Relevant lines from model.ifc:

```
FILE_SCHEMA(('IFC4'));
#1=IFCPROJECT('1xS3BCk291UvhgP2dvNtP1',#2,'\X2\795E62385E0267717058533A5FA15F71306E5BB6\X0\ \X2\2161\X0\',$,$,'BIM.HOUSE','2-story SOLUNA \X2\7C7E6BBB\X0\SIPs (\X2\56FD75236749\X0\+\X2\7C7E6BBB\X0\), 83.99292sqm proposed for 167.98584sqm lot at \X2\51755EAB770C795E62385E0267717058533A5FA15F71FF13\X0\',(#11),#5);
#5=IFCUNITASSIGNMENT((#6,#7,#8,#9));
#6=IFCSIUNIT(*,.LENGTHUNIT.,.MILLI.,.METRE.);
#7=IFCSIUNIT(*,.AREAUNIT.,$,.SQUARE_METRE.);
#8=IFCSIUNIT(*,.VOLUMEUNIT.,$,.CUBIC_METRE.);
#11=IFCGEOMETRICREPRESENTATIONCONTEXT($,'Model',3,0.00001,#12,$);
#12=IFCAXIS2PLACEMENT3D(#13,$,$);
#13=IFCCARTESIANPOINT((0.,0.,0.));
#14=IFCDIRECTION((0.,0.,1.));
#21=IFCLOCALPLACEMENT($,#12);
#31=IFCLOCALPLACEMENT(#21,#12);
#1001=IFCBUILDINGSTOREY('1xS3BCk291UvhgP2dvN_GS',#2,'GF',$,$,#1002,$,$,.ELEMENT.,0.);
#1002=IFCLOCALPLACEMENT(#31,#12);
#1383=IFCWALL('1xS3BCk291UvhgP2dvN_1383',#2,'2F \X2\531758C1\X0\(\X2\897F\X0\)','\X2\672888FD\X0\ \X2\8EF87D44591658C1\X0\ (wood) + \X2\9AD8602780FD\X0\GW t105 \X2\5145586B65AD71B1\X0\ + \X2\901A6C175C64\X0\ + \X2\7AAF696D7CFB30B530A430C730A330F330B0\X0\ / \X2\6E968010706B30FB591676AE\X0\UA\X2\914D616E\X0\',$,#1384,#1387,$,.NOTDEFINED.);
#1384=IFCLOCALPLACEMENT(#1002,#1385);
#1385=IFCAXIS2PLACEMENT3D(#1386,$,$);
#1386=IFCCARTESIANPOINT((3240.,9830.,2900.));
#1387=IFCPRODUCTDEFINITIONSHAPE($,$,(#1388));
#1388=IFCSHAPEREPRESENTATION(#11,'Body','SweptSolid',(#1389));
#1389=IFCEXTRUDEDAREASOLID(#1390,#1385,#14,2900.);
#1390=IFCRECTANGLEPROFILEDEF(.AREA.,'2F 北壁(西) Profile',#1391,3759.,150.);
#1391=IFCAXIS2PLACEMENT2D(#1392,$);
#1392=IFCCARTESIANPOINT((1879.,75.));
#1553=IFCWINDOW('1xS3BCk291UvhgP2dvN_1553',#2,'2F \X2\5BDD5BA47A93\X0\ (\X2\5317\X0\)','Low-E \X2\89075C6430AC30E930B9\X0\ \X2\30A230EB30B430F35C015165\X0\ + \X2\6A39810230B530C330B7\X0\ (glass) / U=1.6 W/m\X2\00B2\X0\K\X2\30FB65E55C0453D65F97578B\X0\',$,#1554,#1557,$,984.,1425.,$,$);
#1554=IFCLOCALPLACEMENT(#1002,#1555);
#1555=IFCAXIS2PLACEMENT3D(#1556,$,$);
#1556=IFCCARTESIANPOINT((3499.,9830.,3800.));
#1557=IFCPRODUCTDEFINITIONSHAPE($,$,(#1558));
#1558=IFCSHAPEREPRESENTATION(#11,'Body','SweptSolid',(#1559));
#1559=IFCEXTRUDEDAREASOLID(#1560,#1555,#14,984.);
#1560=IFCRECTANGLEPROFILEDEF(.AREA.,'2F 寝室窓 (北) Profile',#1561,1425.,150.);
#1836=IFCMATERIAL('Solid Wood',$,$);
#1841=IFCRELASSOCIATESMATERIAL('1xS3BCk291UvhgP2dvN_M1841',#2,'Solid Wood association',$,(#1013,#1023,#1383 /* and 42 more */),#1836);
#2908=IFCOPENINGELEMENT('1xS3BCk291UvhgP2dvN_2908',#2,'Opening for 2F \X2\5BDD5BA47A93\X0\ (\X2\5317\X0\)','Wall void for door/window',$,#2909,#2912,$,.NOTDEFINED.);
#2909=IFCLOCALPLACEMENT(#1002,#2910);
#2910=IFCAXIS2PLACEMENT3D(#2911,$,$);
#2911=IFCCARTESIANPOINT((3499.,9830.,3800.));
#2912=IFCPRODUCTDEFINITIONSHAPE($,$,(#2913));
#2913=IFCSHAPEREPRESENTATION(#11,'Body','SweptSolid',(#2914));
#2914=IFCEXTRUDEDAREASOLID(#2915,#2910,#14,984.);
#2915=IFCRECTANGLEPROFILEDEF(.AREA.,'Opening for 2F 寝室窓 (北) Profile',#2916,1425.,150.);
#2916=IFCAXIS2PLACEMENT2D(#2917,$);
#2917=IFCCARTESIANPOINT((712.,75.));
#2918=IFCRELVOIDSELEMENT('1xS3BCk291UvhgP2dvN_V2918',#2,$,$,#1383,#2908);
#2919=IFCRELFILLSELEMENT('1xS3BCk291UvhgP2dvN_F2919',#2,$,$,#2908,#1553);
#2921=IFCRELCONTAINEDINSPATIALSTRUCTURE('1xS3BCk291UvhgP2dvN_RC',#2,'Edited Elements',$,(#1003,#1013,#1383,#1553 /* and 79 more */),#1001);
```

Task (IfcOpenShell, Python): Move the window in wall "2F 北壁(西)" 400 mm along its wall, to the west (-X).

```python
import ifcopenshell
import ifcopenshell.api.geometry
import ifcopenshell.util.placement
import ifcopenshell.util.unit

model = ifcopenshell.open("model.ifc")
unit_scale = ifcopenshell.util.unit.calculate_unit_scale(model)

window = model.by_guid("1xS3BCk291UvhgP2dvN_1553")
opening = window.FillsVoids[0].RelatingOpeningElement
wall = opening.VoidsElements[0].RelatingBuildingElement

wall_matrix = ifcopenshell.util.placement.get_local_placement(wall.ObjectPlacement)
shift = wall_matrix[:3, 0] * -0.4 / unit_scale
before = ifcopenshell.util.placement.get_local_placement(window.ObjectPlacement)[:3, 3].copy()

# The window is not placed relative to its opening, so move both.
for product in (opening, window):
    matrix = ifcopenshell.util.placement.get_local_placement(product.ObjectPlacement)
    matrix[:3, 3] += shift
    ifcopenshell.api.geometry.edit_object_placement(model, product=product, matrix=matrix, is_si=False)

after = ifcopenshell.util.placement.get_local_placement(window.ObjectPlacement)[:3, 3]
print("window moved by", (after - before).round(3) + 0.0)

model.write("model_v2.ifc")
```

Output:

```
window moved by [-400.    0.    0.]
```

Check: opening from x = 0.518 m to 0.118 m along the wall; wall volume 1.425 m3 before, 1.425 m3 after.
